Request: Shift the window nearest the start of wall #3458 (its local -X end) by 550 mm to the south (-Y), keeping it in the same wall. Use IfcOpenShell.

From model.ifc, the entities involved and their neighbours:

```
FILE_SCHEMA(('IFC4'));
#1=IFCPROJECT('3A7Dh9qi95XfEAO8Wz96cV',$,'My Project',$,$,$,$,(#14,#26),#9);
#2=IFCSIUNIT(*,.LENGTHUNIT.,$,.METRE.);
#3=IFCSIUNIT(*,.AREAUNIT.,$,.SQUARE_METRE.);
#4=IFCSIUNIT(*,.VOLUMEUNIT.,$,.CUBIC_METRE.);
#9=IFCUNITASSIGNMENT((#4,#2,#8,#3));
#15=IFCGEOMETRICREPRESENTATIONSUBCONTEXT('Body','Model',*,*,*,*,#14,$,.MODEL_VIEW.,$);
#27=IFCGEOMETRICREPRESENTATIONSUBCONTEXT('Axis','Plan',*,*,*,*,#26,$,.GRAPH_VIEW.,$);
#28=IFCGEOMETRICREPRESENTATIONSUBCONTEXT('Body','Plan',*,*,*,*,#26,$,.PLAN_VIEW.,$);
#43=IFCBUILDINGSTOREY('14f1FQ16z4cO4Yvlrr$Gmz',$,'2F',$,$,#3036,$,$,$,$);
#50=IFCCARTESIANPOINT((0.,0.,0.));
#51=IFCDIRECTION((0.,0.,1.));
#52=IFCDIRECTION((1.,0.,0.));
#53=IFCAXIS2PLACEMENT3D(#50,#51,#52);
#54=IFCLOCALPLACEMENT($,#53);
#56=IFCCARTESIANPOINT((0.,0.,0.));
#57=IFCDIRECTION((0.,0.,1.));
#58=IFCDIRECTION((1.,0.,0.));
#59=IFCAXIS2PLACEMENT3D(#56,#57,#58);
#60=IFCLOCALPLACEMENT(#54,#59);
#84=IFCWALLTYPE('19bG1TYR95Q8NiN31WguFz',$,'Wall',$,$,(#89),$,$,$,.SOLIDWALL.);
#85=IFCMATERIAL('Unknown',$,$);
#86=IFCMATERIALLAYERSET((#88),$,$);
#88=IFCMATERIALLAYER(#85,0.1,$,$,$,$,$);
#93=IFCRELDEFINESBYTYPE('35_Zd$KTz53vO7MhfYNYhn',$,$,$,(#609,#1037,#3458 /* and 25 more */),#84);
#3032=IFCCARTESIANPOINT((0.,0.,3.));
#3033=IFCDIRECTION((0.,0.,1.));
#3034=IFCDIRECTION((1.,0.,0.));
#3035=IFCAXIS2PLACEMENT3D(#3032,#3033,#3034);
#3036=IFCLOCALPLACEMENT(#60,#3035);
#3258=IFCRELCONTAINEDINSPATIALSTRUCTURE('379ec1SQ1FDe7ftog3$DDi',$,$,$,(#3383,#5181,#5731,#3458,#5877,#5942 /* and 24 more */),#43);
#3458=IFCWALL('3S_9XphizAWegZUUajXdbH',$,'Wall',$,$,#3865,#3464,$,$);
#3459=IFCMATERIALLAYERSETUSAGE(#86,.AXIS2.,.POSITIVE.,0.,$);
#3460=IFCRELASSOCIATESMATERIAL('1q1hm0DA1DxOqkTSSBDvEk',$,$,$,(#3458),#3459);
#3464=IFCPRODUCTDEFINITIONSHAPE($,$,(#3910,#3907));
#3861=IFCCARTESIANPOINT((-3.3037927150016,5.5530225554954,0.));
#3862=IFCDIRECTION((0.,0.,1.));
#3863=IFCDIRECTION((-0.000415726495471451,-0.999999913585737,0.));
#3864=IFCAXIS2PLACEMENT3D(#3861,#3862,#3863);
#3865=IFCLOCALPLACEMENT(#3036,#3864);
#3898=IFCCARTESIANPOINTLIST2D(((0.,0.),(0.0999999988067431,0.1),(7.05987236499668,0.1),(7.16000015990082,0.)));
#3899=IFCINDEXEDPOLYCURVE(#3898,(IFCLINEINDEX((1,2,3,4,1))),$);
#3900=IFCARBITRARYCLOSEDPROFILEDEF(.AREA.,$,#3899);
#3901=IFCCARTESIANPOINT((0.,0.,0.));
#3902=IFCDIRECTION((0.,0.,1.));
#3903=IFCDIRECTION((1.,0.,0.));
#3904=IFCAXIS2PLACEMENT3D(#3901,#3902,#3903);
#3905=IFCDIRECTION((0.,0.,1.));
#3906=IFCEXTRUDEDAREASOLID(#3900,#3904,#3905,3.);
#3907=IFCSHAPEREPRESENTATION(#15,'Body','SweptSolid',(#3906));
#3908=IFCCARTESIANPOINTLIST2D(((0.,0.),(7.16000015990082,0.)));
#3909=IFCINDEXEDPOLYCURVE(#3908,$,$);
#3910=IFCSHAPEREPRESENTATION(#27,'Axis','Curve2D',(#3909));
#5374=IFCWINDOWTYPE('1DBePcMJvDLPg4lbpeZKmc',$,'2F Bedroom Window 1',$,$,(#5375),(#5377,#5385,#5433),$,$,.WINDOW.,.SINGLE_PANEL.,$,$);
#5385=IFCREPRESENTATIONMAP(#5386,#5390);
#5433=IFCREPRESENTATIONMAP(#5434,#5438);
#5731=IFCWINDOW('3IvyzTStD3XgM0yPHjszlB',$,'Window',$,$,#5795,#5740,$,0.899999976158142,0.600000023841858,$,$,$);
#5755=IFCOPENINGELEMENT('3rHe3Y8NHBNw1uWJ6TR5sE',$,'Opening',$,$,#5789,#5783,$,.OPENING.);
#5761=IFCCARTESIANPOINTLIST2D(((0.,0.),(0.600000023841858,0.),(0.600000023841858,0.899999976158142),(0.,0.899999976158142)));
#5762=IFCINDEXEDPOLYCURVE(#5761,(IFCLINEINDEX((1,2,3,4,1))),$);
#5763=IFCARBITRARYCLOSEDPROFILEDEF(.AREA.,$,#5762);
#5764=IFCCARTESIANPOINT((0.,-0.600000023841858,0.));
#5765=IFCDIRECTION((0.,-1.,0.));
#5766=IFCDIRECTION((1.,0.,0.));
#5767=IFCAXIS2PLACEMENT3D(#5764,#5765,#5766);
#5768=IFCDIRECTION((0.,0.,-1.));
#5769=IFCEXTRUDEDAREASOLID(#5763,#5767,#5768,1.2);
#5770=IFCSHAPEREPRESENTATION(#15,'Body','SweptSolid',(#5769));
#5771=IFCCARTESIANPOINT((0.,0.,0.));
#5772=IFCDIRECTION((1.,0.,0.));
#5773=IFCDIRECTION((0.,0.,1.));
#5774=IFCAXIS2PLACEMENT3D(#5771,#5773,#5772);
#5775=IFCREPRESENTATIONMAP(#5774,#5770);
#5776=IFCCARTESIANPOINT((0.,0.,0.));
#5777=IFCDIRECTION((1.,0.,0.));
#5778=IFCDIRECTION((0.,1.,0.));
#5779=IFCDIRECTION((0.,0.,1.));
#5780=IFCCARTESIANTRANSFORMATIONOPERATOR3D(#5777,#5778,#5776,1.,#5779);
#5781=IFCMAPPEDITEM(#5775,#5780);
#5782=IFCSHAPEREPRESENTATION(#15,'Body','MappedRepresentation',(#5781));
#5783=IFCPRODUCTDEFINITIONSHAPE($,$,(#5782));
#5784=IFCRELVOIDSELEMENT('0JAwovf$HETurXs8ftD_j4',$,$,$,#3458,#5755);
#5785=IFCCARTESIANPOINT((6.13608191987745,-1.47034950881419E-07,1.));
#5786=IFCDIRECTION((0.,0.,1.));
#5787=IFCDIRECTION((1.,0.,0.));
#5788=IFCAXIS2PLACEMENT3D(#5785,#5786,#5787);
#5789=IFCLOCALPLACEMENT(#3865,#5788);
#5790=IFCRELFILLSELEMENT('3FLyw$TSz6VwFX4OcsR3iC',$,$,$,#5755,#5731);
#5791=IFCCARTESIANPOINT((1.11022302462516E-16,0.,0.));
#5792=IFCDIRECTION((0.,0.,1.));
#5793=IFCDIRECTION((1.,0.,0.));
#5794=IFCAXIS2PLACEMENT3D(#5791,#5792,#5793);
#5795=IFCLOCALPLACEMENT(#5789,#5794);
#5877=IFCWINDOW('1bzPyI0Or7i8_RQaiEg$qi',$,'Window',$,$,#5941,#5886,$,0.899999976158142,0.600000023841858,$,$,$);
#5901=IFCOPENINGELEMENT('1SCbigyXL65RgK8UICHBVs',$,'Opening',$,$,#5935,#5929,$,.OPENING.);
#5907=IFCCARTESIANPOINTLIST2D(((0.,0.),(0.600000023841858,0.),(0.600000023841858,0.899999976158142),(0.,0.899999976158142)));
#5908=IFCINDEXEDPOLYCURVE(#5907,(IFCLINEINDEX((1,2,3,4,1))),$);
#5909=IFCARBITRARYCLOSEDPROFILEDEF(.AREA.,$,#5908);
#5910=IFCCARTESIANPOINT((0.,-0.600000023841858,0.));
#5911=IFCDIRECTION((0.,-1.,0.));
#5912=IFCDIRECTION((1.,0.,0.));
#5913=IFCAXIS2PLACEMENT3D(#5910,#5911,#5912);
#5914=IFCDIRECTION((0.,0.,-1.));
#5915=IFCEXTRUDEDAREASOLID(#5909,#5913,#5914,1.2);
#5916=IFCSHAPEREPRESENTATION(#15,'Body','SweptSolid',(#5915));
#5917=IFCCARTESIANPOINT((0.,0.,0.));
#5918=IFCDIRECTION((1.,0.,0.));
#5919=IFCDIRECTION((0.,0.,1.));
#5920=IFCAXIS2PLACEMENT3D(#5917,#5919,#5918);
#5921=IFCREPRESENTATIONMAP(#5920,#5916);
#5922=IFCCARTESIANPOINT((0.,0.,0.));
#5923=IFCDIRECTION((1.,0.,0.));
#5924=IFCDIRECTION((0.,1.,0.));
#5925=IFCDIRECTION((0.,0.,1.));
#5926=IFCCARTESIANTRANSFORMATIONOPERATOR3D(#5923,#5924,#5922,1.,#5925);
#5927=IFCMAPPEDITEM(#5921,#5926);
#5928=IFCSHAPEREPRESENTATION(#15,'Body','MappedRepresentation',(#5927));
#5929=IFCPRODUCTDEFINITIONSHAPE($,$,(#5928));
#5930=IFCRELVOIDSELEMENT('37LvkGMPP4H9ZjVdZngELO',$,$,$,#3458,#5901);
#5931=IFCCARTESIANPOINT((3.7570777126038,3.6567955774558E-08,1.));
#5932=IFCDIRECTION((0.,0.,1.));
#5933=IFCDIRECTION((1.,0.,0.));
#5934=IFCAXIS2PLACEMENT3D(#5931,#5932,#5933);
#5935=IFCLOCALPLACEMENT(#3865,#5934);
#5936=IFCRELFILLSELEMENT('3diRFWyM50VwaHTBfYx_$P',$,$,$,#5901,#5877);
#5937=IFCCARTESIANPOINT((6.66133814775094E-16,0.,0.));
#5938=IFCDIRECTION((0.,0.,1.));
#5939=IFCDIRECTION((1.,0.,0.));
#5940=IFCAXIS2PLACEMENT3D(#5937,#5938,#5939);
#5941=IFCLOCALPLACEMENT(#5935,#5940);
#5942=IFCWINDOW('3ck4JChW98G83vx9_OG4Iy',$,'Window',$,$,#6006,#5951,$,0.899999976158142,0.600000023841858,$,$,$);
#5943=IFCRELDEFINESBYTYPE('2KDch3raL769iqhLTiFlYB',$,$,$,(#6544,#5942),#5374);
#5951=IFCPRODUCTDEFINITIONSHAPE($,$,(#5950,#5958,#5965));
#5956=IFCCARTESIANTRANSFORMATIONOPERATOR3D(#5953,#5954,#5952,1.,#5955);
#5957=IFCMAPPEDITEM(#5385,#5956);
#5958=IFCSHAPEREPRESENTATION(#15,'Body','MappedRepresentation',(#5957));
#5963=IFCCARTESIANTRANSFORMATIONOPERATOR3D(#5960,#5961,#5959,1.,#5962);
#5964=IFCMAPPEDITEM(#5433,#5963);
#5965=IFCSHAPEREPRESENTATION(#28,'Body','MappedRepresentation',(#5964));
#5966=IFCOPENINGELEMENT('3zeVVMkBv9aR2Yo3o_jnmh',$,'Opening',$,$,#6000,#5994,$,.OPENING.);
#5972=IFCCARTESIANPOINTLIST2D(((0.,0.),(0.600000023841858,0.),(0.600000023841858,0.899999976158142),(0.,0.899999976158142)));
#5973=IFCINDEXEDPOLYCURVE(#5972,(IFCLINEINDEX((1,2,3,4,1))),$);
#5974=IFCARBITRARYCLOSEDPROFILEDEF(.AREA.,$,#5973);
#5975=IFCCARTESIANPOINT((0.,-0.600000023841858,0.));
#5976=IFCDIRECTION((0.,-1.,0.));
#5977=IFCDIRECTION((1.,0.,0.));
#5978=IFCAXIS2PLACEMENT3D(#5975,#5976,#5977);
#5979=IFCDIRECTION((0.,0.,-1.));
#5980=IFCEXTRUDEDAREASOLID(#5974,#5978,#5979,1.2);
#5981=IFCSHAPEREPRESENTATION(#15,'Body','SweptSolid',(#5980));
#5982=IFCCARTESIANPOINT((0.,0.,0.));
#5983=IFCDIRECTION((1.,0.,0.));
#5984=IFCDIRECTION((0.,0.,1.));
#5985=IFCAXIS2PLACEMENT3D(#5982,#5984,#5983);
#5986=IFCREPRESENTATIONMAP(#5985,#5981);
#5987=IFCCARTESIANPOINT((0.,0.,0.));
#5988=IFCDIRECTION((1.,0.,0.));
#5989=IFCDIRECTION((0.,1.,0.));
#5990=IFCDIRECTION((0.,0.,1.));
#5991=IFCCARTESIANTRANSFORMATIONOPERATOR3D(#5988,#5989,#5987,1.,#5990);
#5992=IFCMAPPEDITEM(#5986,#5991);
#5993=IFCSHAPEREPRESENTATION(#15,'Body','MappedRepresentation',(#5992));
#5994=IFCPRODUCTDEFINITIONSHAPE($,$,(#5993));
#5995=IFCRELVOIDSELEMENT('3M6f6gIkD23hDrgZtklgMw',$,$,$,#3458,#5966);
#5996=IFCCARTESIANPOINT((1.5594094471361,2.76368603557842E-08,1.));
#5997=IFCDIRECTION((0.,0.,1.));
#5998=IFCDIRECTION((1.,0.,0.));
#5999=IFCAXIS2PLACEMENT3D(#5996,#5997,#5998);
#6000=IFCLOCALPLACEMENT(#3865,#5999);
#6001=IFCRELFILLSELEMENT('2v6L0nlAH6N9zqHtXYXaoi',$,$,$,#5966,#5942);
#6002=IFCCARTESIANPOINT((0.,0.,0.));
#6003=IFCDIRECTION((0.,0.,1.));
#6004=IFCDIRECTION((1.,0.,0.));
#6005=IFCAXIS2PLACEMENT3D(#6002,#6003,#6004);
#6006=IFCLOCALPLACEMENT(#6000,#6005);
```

```python
import ifcopenshell
import ifcopenshell.api.geometry
import ifcopenshell.util.placement
import ifcopenshell.util.unit

model = ifcopenshell.open("model.ifc")
unit_scale = ifcopenshell.util.unit.calculate_unit_scale(model)

window = model.by_guid("3ck4JChW98G83vx9_OG4Iy")
opening = window.FillsVoids[0].RelatingOpeningElement
wall = opening.VoidsElements[0].RelatingBuildingElement

wall_matrix = ifcopenshell.util.placement.get_local_placement(wall.ObjectPlacement)
shift = wall_matrix[:3, 0] * 0.55 / unit_scale
before = ifcopenshell.util.placement.get_local_placement(window.ObjectPlacement)[:3, 3].copy()

# The window is placed relative to its opening, so it follows when the opening moves.
matrix = ifcopenshell.util.placement.get_local_placement(opening.ObjectPlacement)
matrix[:3, 3] += shift
ifcopenshell.api.geometry.edit_object_placement(
    model, product=opening, matrix=matrix, is_si=False, should_transform_children=True
)

after = ifcopenshell.util.placement.get_local_placement(window.ObjectPlacement)[:3, 3]
print("window moved by", (after - before).round(3) + 0.0)

model.write("model_v2.ifc")
```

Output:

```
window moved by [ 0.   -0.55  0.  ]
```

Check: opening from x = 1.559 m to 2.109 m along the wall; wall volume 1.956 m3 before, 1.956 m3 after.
